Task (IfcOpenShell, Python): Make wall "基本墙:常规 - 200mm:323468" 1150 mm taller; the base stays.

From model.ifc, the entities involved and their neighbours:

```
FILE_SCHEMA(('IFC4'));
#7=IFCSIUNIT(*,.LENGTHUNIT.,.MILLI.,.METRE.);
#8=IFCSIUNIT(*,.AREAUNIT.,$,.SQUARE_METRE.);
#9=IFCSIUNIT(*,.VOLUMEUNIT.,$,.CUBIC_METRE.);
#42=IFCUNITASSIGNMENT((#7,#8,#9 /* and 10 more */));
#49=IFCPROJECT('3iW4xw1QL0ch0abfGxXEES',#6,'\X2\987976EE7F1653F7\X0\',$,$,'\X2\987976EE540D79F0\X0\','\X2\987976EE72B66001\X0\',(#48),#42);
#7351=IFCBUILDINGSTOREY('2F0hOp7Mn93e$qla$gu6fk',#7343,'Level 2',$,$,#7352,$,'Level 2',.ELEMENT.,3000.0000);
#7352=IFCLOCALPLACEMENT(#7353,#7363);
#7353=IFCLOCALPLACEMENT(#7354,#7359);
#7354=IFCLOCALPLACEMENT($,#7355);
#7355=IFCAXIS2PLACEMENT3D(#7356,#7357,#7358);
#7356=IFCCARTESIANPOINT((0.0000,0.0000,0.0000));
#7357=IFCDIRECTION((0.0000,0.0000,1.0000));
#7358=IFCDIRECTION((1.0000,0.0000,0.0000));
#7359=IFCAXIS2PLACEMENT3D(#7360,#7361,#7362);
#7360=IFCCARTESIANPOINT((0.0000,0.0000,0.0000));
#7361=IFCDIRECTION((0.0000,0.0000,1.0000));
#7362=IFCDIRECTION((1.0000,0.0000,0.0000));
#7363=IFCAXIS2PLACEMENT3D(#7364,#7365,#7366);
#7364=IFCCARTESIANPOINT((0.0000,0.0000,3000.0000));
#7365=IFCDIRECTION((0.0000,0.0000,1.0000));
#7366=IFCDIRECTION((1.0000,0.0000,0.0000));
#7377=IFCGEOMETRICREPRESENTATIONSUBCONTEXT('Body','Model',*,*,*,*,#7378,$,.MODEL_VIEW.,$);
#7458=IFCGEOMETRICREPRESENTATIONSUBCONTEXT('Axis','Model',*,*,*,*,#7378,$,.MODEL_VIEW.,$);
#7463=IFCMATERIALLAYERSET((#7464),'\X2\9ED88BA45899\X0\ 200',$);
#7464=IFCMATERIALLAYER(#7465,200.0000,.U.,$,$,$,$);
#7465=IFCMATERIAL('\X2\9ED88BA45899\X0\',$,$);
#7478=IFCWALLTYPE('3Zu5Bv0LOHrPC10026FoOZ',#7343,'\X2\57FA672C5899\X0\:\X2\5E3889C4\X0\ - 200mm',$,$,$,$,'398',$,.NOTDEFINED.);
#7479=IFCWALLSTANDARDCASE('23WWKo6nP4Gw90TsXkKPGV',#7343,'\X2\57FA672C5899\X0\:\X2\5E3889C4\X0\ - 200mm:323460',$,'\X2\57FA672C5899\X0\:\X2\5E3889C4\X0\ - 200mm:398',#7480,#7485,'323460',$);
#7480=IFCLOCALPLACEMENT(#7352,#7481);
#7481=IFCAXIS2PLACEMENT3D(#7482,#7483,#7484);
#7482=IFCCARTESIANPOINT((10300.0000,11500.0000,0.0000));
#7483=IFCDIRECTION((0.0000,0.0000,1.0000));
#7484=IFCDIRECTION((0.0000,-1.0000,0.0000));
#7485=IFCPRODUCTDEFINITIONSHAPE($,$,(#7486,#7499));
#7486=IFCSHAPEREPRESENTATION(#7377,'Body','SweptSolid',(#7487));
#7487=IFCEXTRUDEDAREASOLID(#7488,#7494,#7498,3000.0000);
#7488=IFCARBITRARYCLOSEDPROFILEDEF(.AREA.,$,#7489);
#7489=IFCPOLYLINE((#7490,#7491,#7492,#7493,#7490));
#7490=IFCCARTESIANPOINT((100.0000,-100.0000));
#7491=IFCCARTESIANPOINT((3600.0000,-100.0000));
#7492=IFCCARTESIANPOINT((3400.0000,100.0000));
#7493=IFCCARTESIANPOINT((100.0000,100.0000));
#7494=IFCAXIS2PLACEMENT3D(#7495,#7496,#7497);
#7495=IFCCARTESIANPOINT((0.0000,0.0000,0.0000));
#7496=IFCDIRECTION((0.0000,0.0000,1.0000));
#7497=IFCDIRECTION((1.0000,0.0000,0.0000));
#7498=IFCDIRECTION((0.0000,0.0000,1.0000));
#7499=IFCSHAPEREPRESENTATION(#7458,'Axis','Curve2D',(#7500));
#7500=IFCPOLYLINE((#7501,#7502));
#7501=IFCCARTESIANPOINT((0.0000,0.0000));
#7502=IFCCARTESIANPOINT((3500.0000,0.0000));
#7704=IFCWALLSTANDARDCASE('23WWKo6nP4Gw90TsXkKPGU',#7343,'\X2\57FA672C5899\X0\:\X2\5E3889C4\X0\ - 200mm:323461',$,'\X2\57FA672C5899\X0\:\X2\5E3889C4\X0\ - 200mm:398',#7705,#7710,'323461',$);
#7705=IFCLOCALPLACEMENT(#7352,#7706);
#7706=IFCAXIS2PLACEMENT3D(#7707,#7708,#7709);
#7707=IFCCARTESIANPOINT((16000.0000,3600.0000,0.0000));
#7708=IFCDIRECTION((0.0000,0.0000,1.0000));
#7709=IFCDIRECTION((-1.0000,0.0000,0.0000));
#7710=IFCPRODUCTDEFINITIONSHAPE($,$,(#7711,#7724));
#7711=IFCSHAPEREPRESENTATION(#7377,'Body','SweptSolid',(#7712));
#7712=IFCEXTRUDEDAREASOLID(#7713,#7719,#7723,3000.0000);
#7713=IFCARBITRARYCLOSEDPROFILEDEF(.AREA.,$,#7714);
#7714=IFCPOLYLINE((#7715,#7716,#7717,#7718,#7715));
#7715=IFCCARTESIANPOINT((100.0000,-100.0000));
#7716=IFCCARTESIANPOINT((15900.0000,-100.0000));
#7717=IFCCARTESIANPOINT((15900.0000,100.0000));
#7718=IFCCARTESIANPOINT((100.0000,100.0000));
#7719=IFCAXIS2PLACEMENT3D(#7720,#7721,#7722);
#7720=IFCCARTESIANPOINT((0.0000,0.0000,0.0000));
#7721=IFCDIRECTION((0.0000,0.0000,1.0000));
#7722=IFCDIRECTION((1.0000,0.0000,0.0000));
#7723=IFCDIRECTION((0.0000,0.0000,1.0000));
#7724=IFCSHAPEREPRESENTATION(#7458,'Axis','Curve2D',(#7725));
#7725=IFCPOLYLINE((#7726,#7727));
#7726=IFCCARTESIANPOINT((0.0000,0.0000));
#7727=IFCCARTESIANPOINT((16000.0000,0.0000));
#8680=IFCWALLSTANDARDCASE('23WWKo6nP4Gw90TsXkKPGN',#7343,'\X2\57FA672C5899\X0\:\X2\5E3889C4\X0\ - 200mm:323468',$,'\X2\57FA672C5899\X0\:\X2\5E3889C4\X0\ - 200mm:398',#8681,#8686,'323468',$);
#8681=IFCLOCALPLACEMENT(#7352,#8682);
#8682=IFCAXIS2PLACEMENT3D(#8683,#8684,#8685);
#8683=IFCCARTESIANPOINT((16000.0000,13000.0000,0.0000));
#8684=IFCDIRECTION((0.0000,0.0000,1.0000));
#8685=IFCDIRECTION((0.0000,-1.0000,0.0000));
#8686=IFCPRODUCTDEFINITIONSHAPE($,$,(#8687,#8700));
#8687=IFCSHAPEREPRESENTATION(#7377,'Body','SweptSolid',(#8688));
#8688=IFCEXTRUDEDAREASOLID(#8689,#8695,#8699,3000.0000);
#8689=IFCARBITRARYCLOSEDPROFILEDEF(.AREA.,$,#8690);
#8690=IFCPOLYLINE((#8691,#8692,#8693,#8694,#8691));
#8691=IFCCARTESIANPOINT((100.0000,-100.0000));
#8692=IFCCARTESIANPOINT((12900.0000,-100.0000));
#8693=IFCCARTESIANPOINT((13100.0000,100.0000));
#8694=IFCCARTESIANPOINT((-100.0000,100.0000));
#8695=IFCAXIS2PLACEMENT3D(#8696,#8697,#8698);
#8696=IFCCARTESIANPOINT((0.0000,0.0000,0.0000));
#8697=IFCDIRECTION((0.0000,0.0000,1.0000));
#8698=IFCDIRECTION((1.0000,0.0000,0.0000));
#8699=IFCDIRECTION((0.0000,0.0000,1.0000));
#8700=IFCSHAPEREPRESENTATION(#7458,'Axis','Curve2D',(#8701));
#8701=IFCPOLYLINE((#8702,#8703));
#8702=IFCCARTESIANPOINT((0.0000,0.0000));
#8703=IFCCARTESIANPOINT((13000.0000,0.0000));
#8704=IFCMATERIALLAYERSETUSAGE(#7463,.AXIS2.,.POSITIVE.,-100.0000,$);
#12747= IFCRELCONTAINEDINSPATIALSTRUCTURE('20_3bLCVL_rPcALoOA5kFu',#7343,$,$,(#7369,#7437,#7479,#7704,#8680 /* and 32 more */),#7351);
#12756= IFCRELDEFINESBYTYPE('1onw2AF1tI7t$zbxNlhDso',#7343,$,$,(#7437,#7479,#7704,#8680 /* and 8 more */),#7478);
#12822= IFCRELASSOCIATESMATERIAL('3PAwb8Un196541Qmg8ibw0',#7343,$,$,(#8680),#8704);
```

```python
import ifcopenshell
import ifcopenshell.geom
import ifcopenshell.util.representation
import ifcopenshell.util.shape

model = ifcopenshell.open("model.ifc")
settings = ifcopenshell.geom.settings()


def volume(element):
    """Net volume in cubic metres, openings subtracted."""
    shape = ifcopenshell.geom.create_shape(settings, element)
    return ifcopenshell.util.shape.get_volume(shape.geometry)


wall = model.by_id(8680)
before = volume(wall)

body = ifcopenshell.util.representation.get_representation(wall, "Model", "Body")
solid = body.Items[0]
old_height = solid.Depth
solid.Depth += 1150.0
after = volume(wall)

print(f"height {old_height:g} -> {solid.Depth:g}, volume {before:.3f} -> {after:.3f} m3")

model.write("model_rev.ifc")
```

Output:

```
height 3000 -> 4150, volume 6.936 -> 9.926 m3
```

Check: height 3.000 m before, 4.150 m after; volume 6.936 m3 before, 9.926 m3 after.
